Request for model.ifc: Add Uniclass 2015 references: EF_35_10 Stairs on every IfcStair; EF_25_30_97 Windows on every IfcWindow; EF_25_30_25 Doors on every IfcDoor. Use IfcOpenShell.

First a look at what the model holds.

```python
import ifcopenshell

model = ifcopenshell.open("model.ifc")
print(model.schema)
print("classifications:", [c.Name for c in model.by_type("IfcClassification")])
for ifc_class in ("IfcDoor", "IfcRoof", "IfcStair", "IfcWall", "IfcWindow"):
    print(ifc_class, len(model.by_type(ifc_class)))
```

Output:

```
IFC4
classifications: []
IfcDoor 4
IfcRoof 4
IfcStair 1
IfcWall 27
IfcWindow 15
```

```python
import ifcopenshell
import ifcopenshell.api.classification

model = ifcopenshell.open("model.ifc")

system = ifcopenshell.api.classification.add_classification(model, classification="Uniclass 2015")

codes = {
    "IfcStair": ("EF_35_10", "Stairs"),
    "IfcWindow": ("EF_25_30_97", "Windows"),
    "IfcDoor": ("EF_25_30_25", "Doors"),
}
for ifc_class, (code, name) in codes.items():
    products = model.by_type(ifc_class)
    ifcopenshell.api.classification.add_reference(
        model, products=products, classification=system, identification=code, name=name
    )
    print(code, len(products))

model.write("model_v2.ifc")
```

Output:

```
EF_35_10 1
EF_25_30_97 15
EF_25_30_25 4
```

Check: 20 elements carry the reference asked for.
